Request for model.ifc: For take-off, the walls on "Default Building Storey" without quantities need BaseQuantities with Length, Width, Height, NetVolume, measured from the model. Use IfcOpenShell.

First a look at what the model holds.

```python
import ifcopenshell
import ifcopenshell.util.element
import ifcopenshell.util.unit

model = ifcopenshell.open("model.ifc")
print(model.schema)
for unit_type in ("LENGTHUNIT", "AREAUNIT", "VOLUMEUNIT"):
    print(unit_type, ifcopenshell.util.unit.calculate_unit_scale(model, unit_type))
storey = next(s for s in model.by_type("IfcBuildingStorey") if s.Name == "Default Building Storey")
walls = [e for e in ifcopenshell.util.element.get_decomposition(storey) if e.is_a("IfcWall")]
for e in sorted(walls, key=lambda e: e.id()):
    print(e.id(), e.is_a(), e.Name, list(ifcopenshell.util.element.get_psets(e, qtos_only=True)), sep=" | ")
```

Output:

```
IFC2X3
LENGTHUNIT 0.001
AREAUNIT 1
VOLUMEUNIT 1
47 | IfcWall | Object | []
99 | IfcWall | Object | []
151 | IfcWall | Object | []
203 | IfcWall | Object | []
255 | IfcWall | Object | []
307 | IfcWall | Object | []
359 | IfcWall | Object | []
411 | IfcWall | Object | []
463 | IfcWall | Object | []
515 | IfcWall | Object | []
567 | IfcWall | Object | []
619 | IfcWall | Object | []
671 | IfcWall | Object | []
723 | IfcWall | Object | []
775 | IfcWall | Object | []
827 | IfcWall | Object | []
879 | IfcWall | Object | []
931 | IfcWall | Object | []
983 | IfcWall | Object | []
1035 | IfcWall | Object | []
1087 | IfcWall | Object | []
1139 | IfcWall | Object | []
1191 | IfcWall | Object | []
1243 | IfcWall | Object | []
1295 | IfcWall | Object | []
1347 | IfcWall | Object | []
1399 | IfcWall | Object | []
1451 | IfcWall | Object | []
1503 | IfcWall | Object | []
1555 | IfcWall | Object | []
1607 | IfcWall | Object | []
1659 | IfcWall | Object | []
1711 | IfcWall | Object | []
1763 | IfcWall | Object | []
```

```python
import ifcopenshell
import ifcopenshell.api.pset
import ifcopenshell.geom
import ifcopenshell.util.element
import ifcopenshell.util.shape
import ifcopenshell.util.unit

model = ifcopenshell.open("model.ifc")
unit_scale = ifcopenshell.util.unit.calculate_unit_scale(model)
volume_scale = ifcopenshell.util.unit.calculate_unit_scale(model, "VOLUMEUNIT")
settings = ifcopenshell.geom.settings()

storey = next(s for s in model.by_type("IfcBuildingStorey") if s.Name == "Default Building Storey")
walls = [e for e in ifcopenshell.util.element.get_decomposition(storey) if e.is_a("IfcWall")]

for e in sorted(walls, key=lambda e: e.id()):
    if ifcopenshell.util.element.get_psets(e, qtos_only=True, should_inherit=False):
        continue
    # Geometry comes back in metres, in the element's own axes.
    shape = ifcopenshell.geom.create_shape(settings, e)
    values = {
        "Length": ifcopenshell.util.shape.get_x(shape.geometry) / unit_scale,
        "Width": ifcopenshell.util.shape.get_y(shape.geometry) / unit_scale,
        "Height": ifcopenshell.util.shape.get_z(shape.geometry) / unit_scale,
        "NetVolume": ifcopenshell.util.shape.get_volume(shape.geometry) / volume_scale,
    }
    qto = ifcopenshell.api.pset.add_qto(model, product=e, name="BaseQuantities")
    ifcopenshell.api.pset.edit_qto(model, qto=qto, properties=values)
    print(e.id(), {k: round(v, 3) for k, v in values.items()})

model.write("model-out.ifc")
```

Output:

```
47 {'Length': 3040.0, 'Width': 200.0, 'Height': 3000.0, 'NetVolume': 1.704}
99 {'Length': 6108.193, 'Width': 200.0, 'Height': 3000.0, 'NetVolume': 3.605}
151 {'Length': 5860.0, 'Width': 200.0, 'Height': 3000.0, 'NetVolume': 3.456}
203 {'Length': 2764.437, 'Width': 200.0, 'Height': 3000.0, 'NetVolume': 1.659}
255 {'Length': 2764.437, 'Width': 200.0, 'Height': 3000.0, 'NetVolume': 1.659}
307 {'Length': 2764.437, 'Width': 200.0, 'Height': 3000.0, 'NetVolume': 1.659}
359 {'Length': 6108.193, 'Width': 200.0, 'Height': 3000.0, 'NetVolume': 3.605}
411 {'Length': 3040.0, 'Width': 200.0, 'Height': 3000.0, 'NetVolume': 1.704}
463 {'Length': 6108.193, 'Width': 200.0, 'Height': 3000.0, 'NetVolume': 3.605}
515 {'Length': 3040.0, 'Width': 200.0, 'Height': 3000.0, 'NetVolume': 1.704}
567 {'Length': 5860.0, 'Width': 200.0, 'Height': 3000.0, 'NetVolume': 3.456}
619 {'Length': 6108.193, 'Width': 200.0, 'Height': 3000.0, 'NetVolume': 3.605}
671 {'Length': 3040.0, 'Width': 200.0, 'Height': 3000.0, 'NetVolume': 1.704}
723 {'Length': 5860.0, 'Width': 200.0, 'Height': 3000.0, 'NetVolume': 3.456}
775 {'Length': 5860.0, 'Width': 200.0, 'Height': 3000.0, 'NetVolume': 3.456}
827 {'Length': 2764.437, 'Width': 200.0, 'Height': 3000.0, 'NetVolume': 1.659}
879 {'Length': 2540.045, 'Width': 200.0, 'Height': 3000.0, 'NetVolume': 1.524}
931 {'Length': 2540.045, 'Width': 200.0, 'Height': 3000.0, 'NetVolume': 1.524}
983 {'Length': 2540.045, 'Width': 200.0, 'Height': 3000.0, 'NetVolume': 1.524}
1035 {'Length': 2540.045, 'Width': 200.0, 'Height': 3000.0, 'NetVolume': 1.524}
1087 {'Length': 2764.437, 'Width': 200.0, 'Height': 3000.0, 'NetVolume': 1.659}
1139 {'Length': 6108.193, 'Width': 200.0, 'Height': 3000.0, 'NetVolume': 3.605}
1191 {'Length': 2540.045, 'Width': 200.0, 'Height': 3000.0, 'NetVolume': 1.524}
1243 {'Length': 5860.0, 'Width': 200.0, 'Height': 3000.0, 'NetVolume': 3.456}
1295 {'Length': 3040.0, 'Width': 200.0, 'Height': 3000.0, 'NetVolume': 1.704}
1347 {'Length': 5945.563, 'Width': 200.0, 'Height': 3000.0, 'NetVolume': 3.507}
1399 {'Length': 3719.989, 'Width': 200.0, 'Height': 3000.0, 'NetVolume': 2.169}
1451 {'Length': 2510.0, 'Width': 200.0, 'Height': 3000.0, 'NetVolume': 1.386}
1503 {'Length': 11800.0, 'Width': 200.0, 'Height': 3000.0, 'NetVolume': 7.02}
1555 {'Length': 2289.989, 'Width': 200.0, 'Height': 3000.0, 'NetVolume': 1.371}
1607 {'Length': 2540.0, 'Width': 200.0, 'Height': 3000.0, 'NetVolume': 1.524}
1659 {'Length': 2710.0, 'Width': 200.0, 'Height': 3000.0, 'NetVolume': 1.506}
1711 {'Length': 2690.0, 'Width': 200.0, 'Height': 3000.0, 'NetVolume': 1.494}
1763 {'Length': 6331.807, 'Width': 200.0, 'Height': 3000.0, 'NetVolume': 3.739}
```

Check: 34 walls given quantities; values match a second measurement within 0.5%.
